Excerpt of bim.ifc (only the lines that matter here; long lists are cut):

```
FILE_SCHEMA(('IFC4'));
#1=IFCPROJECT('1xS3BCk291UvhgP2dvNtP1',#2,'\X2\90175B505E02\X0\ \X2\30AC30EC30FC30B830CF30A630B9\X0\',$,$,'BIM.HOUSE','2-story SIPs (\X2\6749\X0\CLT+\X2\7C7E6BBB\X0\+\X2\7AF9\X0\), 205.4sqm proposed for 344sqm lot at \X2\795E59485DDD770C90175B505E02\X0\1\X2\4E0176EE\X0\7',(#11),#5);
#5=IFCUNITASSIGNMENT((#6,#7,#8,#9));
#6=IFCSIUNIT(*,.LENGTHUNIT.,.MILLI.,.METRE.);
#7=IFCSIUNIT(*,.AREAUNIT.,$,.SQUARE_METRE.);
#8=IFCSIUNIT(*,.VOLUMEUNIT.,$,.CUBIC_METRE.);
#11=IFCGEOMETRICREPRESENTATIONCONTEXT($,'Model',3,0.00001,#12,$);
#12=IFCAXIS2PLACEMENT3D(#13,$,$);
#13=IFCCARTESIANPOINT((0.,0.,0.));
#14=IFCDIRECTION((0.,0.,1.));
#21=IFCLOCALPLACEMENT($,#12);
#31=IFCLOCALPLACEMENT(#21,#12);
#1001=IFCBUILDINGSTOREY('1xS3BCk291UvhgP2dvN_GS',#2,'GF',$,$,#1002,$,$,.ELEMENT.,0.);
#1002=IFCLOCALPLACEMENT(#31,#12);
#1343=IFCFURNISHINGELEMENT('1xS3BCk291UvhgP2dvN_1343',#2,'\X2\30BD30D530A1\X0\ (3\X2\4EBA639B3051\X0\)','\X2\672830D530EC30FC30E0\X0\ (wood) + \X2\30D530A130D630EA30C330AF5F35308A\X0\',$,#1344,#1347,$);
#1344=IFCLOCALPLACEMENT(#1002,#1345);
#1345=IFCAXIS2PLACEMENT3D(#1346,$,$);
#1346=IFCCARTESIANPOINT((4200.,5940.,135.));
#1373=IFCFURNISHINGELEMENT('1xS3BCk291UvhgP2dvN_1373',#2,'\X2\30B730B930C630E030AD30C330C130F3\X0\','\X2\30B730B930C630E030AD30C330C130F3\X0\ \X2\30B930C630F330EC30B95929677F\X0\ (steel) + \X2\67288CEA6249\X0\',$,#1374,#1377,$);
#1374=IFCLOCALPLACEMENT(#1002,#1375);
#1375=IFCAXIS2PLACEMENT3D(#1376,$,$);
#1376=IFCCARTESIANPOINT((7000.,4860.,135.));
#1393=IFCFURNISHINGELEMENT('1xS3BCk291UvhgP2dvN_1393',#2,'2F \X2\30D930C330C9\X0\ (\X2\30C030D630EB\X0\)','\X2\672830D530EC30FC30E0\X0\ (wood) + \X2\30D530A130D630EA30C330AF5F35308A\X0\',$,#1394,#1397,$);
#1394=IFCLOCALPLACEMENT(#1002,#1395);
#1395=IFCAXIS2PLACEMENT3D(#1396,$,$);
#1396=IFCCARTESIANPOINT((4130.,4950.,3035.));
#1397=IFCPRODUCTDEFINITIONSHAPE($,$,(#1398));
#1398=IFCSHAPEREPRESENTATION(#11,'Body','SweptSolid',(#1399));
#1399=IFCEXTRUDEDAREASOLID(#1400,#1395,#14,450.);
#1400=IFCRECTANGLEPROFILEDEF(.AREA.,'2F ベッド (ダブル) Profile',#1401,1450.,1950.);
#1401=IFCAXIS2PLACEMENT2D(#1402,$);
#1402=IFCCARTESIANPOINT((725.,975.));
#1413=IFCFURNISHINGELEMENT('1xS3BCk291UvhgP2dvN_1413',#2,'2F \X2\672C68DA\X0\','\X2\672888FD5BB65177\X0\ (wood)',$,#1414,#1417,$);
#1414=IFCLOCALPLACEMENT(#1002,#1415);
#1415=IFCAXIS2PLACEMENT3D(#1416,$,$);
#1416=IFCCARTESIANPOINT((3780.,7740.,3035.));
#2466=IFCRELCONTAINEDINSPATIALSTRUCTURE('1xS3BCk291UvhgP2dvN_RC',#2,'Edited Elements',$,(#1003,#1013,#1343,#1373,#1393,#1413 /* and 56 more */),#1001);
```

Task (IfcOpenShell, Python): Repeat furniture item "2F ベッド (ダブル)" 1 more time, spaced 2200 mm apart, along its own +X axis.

```python
import ifcopenshell
import ifcopenshell.api.geometry
import ifcopenshell.api.root
import ifcopenshell.util.element
import ifcopenshell.util.placement

model = ifcopenshell.open("bim.ifc")


def reuse_history(source, copy):
    """copy_class also copies each property set's owner history, people and application; keep the originals."""
    for rel in copy.IsDefinedBy:
        if rel.is_a("IfcRelDefinesByProperties") and (history := rel.RelatingPropertyDefinition.OwnerHistory):
            rel.RelatingPropertyDefinition.OwnerHistory = source.OwnerHistory
            ifcopenshell.util.element.remove_deep2(model, history)


source = model.by_guid("1xS3BCk291UvhgP2dvN_1393")
base = ifcopenshell.util.placement.get_local_placement(source.ObjectPlacement)
step = base[:3, 0] * 2200.0

for i in range(1, 2):
    copy = ifcopenshell.api.root.copy_class(model, product=source)
    copy.Representation = ifcopenshell.util.element.copy_deep(
        model, source.Representation, exclude=["IfcGeometricRepresentationContext", "IfcRepresentationMap"]
    )
    reuse_history(source, copy)
    matrix = base.copy()
    matrix[:3, 3] += i * step
    print("added at", matrix[:3, 3].round(3) + 0.0)
    ifcopenshell.api.geometry.edit_object_placement(model, product=copy, matrix=matrix, is_si=False)

model.write("bim-out.ifc")
```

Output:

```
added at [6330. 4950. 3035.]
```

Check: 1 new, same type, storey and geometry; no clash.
